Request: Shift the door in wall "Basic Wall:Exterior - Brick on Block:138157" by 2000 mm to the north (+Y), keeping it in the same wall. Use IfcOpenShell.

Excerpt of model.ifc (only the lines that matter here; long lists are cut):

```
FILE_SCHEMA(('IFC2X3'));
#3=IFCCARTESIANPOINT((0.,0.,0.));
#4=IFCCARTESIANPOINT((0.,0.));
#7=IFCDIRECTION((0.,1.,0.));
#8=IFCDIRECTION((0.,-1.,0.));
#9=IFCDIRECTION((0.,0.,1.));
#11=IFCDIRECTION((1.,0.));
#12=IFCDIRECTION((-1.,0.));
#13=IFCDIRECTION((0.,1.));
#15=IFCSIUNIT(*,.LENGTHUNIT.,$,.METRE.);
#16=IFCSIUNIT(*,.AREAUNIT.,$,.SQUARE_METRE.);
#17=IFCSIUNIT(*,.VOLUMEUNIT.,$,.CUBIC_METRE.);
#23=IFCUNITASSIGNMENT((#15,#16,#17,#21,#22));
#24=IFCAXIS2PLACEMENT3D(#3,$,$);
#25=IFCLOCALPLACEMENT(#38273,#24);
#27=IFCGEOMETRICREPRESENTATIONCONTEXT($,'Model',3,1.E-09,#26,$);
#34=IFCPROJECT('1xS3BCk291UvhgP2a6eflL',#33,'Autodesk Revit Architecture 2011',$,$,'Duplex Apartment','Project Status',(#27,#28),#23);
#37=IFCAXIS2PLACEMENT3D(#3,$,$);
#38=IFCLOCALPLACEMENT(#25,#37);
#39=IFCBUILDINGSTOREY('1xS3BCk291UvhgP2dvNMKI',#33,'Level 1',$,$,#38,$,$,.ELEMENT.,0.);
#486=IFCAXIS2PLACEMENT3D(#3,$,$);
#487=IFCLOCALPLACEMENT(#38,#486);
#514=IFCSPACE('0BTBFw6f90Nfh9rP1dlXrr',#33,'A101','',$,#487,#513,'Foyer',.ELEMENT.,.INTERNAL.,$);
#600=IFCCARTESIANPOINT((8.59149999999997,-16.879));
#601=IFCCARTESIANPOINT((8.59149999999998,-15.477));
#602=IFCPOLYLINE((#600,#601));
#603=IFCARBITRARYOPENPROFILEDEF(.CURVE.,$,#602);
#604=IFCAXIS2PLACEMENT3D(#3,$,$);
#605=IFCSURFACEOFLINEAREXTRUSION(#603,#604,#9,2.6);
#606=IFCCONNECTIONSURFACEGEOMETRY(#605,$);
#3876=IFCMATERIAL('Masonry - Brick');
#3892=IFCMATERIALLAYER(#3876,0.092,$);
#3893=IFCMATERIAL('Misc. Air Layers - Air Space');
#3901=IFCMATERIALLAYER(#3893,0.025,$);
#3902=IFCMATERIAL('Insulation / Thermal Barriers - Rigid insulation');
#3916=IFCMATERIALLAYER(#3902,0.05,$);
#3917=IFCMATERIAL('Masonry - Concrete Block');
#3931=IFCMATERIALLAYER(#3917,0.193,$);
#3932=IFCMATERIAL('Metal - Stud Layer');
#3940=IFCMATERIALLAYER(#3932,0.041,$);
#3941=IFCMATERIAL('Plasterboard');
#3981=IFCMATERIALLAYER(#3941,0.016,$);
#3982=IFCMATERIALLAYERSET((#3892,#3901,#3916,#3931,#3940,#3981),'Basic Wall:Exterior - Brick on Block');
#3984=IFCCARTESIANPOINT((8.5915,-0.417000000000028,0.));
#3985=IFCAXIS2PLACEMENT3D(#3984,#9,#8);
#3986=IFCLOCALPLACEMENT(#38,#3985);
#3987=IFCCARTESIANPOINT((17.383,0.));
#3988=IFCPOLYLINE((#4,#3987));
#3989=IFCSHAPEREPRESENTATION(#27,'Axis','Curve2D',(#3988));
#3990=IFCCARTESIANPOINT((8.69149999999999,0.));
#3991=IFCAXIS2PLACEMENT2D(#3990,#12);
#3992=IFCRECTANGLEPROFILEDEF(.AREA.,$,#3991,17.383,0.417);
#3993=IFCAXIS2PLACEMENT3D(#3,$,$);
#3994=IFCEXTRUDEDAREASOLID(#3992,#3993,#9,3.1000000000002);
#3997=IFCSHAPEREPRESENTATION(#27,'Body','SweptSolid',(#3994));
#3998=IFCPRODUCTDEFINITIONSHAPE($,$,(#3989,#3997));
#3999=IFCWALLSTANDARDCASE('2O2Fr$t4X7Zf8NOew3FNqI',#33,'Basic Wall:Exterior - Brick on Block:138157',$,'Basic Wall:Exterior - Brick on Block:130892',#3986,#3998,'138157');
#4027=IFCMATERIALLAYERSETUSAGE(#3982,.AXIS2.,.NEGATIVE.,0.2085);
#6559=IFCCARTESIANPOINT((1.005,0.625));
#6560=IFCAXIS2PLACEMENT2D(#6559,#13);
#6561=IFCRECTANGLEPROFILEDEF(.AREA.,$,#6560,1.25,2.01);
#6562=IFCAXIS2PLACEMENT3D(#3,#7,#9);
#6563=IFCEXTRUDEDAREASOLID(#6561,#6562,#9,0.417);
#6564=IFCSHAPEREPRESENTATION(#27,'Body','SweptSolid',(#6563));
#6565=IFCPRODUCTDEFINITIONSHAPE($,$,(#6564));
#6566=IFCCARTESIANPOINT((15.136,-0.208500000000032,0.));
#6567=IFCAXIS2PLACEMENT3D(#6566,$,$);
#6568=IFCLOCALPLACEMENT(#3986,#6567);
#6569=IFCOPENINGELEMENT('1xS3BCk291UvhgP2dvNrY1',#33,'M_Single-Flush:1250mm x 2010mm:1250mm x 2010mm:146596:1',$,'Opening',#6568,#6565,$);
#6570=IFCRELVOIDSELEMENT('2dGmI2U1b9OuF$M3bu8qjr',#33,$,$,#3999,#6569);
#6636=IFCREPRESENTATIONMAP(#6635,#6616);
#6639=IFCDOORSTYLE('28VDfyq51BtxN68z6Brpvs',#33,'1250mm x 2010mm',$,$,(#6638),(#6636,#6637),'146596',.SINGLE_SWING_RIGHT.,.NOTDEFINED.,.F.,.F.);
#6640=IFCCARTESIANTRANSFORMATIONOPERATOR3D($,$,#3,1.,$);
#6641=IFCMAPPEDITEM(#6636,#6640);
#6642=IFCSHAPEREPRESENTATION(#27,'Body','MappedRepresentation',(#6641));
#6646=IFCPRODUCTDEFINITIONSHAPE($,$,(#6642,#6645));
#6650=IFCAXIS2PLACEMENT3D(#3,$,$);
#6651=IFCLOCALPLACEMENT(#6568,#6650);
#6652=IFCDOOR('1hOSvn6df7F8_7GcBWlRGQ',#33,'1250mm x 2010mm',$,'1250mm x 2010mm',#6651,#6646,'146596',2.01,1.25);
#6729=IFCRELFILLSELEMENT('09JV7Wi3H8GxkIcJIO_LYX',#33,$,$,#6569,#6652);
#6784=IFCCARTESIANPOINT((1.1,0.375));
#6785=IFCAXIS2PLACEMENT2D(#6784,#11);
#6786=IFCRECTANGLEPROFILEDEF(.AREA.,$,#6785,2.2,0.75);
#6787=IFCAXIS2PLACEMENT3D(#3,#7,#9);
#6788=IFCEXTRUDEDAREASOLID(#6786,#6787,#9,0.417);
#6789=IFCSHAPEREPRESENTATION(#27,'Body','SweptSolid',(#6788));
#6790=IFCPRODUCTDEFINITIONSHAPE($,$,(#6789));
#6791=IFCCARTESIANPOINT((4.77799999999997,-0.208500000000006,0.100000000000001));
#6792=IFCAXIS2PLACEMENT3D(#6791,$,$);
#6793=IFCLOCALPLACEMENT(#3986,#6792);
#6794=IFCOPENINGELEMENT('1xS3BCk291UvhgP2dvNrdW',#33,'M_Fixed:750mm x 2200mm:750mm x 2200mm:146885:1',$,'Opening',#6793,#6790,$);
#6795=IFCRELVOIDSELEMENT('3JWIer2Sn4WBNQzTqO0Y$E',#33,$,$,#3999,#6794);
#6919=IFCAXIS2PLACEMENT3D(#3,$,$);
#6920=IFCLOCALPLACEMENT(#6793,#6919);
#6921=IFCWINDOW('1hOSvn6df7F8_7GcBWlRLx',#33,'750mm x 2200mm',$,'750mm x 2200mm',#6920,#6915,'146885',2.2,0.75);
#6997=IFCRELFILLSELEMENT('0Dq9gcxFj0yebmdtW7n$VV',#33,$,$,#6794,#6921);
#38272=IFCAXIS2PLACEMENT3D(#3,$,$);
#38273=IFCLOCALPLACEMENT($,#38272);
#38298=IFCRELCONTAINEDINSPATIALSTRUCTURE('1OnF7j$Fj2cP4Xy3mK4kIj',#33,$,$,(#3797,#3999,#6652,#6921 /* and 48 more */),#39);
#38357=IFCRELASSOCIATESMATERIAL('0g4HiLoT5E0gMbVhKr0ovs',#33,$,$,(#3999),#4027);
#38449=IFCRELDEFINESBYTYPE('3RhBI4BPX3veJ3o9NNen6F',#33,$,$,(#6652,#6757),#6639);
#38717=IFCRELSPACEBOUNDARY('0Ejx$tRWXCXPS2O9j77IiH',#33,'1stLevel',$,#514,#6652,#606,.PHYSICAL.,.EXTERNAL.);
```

```python
import numpy as np
import ifcopenshell
import ifcopenshell.api.geometry
import ifcopenshell.util.placement
import ifcopenshell.util.unit

model = ifcopenshell.open("model.ifc")
unit_scale = ifcopenshell.util.unit.calculate_unit_scale(model)

door = model.by_guid("1hOSvn6df7F8_7GcBWlRGQ")
opening = door.FillsVoids[0].RelatingOpeningElement
wall = opening.VoidsElements[0].RelatingBuildingElement

wall_matrix = ifcopenshell.util.placement.get_local_placement(wall.ObjectPlacement)
shift = wall_matrix[:3, 0] * -2 / unit_scale
before = ifcopenshell.util.placement.get_local_placement(door.ObjectPlacement)[:3, 3].copy()

# The door is placed relative to its opening, so it follows when the opening moves.
matrix = ifcopenshell.util.placement.get_local_placement(opening.ObjectPlacement)
matrix[:3, 3] += shift
ifcopenshell.api.geometry.edit_object_placement(
    model, product=opening, matrix=matrix, is_si=False, should_transform_children=True
)

# Space boundary surfaces are stored in each space's coordinates; move them too.
for rel in door.ProvidesBoundaries:
    if not rel.ConnectionGeometry:
        continue
    surface = rel.ConnectionGeometry.SurfaceOnRelatingElement
    space_matrix = ifcopenshell.util.placement.get_local_placement(rel.RelatingSpace.ObjectPlacement)
    point = np.array(surface.Position.Location.Coordinates) + space_matrix[:3, :3].T @ shift
    surface.Position = model.createIfcAxis2Placement3D(
        model.createIfcCartesianPoint(point.tolist()), surface.Position.Axis, surface.Position.RefDirection
    )

after = ifcopenshell.util.placement.get_local_placement(door.ObjectPlacement)[:3, 3]
print("door moved by", (after - before).round(3) + 0.0)

model.write("model_edited.ifc")
```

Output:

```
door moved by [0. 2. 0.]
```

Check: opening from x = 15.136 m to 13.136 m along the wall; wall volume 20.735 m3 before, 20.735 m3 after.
